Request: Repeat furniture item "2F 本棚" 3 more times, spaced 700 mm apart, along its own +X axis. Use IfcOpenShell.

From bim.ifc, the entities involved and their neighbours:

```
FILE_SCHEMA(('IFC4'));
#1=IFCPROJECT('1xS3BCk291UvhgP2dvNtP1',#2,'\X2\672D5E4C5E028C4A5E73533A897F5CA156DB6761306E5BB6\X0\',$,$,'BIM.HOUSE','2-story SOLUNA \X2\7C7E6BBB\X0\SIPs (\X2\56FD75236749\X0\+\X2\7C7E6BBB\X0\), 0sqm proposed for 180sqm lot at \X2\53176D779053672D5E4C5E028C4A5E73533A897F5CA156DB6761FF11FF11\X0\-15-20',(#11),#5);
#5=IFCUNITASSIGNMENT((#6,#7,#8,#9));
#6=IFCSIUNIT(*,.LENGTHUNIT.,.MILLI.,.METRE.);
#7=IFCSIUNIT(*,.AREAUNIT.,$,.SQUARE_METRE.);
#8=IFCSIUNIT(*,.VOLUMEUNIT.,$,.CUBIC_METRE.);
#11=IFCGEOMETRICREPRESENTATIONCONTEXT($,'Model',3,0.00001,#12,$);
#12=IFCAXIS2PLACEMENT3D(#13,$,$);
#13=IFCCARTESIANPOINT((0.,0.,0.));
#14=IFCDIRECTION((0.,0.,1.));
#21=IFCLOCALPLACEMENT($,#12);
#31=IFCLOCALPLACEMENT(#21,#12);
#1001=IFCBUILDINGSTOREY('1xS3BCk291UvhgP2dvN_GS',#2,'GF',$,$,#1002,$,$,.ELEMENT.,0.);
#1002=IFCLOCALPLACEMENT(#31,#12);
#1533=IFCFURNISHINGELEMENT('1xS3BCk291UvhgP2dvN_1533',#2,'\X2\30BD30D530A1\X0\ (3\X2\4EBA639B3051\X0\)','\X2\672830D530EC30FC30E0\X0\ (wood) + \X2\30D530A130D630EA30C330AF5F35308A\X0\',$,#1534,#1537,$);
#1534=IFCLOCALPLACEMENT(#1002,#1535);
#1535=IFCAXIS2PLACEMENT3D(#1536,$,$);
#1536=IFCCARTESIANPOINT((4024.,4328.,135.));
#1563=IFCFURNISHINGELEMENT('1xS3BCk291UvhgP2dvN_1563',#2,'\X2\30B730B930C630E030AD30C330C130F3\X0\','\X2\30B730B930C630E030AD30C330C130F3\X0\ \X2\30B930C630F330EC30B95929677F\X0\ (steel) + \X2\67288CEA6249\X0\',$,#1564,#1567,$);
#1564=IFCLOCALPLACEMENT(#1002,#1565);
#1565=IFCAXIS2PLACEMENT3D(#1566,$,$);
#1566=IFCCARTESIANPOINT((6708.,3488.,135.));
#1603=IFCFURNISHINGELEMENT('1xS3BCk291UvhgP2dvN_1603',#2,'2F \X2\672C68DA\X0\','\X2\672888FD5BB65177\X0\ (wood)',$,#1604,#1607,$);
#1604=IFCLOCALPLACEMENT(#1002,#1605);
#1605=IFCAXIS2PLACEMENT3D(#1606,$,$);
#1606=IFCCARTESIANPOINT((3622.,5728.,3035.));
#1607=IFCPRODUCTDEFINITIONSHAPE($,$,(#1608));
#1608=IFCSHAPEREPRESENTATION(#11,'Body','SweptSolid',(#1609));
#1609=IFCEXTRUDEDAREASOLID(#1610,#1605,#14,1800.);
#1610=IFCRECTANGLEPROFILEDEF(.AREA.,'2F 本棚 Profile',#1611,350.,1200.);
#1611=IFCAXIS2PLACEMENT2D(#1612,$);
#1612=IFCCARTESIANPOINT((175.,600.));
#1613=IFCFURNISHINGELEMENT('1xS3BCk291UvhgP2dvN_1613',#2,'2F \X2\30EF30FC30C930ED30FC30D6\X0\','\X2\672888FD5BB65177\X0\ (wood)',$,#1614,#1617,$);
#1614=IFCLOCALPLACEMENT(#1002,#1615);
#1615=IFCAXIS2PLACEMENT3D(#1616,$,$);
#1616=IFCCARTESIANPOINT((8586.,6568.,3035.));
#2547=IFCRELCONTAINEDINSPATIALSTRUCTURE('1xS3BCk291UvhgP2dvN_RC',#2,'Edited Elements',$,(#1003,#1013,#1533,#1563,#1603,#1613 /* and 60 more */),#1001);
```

```python
import ifcopenshell
import ifcopenshell.api.geometry
import ifcopenshell.api.root
import ifcopenshell.util.element
import ifcopenshell.util.placement
import ifcopenshell.util.unit

model = ifcopenshell.open("bim.ifc")
unit_scale = ifcopenshell.util.unit.calculate_unit_scale(model)


def reuse_history(source, copy):
    """copy_class also copies each property set's owner history, people and application; keep the originals."""
    for rel in copy.IsDefinedBy:
        if rel.is_a("IfcRelDefinesByProperties") and (history := rel.RelatingPropertyDefinition.OwnerHistory):
            rel.RelatingPropertyDefinition.OwnerHistory = source.OwnerHistory
            ifcopenshell.util.element.remove_deep2(model, history)


source = model.by_guid("1xS3BCk291UvhgP2dvN_1603")
base = ifcopenshell.util.placement.get_local_placement(source.ObjectPlacement)
step = base[:3, 0] * 0.7 / unit_scale

for i in range(1, 4):
    copy = ifcopenshell.api.root.copy_class(model, product=source)
    copy.Representation = ifcopenshell.util.element.copy_deep(
        model, source.Representation, exclude=["IfcGeometricRepresentationContext", "IfcRepresentationMap"]
    )
    reuse_history(source, copy)
    matrix = base.copy()
    matrix[:3, 3] += i * step
    print("added at", matrix[:3, 3].round(3) + 0.0)
    ifcopenshell.api.geometry.edit_object_placement(model, product=copy, matrix=matrix, is_si=False)

model.write("bim_v2.ifc")
```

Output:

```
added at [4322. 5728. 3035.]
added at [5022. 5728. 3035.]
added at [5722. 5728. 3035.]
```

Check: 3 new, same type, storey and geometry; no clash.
